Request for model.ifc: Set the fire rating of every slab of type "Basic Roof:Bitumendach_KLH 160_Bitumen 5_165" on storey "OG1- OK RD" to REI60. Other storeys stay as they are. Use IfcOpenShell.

First a look at what the model holds.

```python
import ifcopenshell
import ifcopenshell.util.element

model = ifcopenshell.open("model.ifc")
print(model.schema)
storey = next(s for s in model.by_type("IfcBuildingStorey") if s.Name == "OG1- OK RD")
slabs = [e for e in ifcopenshell.util.element.get_decomposition(storey) if e.is_a("IfcSlab")]
seen = {}
for e in slabs:
    element_type = ifcopenshell.util.element.get_type(e)
    key = (element_type.Name if element_type != e and element_type else None, ifcopenshell.util.element.get_pset(e, "Pset_SlabCommon", "FireRating"))
    seen[key] = seen.get(key, 0) + 1
for (name, value), count in sorted(seen.items(), key=str):
    print(count, "x", name, "|", value)
```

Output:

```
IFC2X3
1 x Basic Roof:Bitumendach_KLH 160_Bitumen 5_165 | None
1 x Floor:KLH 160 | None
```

```python
import ifcopenshell
import ifcopenshell.api.pset
import ifcopenshell.util.element

model = ifcopenshell.open("model.ifc")

storey = next(s for s in model.by_type("IfcBuildingStorey") if s.Name == "OG1- OK RD")
slabs = [e for e in ifcopenshell.util.element.get_decomposition(storey) if e.is_a("IfcSlab")]

count = 0
for e in slabs:
    element_type = ifcopenshell.util.element.get_type(e)
    if element_type in (None, e) or element_type.Name != "Basic Roof:Bitumendach_KLH 160_Bitumen 5_165":
        continue
    # add_pset returns the element's existing set when there is one.
    pset = ifcopenshell.api.pset.add_pset(model, product=e, name="Pset_SlabCommon")
    ifcopenshell.api.pset.edit_pset(model, pset=pset, properties={"FireRating": "REI60"})
    count += 1

print(count, "slabs updated")

model.write("model_rev.ifc")
```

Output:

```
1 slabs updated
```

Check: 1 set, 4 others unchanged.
